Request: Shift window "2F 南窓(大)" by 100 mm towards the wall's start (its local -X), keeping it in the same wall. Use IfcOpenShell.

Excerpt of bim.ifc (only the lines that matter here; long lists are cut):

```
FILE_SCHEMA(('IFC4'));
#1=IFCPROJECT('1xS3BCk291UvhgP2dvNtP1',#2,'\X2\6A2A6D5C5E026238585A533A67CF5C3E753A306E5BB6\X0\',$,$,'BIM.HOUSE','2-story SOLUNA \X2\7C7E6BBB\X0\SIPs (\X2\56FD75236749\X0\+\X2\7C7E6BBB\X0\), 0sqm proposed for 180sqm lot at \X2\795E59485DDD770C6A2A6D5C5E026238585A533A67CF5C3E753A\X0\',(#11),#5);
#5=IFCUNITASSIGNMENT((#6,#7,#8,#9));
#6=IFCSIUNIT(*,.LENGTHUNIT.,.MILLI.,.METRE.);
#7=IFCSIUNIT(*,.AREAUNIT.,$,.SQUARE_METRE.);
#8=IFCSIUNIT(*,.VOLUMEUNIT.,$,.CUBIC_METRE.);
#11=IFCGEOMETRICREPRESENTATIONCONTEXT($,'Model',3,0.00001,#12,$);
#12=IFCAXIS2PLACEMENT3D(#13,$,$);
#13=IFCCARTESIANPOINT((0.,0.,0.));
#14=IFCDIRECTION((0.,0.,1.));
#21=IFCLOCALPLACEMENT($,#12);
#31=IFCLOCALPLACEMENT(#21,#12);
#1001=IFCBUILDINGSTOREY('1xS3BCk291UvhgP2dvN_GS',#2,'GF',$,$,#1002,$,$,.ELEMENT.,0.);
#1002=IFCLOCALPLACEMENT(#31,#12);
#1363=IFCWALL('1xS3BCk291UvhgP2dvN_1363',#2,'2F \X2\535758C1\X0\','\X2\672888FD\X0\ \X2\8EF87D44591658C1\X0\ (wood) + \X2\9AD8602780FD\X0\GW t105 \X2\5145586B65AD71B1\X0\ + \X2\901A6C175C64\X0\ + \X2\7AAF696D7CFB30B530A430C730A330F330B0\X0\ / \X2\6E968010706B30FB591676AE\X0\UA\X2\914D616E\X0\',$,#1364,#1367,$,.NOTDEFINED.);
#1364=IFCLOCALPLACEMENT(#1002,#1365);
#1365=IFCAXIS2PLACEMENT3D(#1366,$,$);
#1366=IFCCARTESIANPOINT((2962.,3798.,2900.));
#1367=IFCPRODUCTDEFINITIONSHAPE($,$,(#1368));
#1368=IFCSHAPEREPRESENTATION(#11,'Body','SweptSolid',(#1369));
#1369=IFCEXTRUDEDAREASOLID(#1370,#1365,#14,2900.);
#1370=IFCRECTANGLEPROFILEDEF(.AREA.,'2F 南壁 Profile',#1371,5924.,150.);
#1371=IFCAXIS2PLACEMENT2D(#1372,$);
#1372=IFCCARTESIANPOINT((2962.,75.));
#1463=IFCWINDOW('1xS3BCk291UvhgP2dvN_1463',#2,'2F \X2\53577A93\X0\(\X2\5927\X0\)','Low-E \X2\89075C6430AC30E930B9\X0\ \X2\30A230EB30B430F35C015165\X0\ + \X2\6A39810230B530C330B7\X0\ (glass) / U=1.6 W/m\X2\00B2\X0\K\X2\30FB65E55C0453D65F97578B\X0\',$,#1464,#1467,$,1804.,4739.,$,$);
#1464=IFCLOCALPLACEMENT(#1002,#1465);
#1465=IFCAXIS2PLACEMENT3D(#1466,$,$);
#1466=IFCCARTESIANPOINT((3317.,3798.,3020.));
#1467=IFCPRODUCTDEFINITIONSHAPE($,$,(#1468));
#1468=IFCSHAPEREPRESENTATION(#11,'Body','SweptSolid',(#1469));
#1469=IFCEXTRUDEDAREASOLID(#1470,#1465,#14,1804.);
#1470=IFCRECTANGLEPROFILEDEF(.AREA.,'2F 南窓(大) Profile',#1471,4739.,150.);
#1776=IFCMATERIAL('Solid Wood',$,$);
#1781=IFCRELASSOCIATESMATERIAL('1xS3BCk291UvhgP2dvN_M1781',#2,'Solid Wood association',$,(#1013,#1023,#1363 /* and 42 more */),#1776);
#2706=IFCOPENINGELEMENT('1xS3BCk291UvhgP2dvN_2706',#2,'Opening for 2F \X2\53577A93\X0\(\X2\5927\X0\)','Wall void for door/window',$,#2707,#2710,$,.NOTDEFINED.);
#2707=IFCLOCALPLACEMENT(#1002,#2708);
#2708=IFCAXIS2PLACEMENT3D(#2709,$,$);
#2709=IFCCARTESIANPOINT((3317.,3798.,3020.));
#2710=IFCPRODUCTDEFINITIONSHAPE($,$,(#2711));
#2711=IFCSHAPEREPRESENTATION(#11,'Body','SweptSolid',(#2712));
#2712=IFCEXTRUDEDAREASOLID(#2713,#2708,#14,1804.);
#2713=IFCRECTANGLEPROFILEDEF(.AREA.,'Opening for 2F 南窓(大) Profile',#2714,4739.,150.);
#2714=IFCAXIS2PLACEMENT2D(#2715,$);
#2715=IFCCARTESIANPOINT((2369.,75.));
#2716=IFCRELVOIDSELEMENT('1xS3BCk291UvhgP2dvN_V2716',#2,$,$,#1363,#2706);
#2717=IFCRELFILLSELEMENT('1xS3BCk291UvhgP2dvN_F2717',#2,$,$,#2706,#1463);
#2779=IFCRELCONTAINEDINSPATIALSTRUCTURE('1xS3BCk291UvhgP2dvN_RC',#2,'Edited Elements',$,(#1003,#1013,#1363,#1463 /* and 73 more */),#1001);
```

```python
import ifcopenshell
import ifcopenshell.api.geometry
import ifcopenshell.util.placement
import ifcopenshell.util.unit

model = ifcopenshell.open("bim.ifc")
unit_scale = ifcopenshell.util.unit.calculate_unit_scale(model)

window = model.by_id(1463)
opening = window.FillsVoids[0].RelatingOpeningElement
wall = opening.VoidsElements[0].RelatingBuildingElement

wall_matrix = ifcopenshell.util.placement.get_local_placement(wall.ObjectPlacement)
shift = wall_matrix[:3, 0] * -0.1 / unit_scale
before = ifcopenshell.util.placement.get_local_placement(window.ObjectPlacement)[:3, 3].copy()

# The window is not placed relative to its opening, so move both.
for product in (opening, window):
    matrix = ifcopenshell.util.placement.get_local_placement(product.ObjectPlacement)
    matrix[:3, 3] += shift
    ifcopenshell.api.geometry.edit_object_placement(model, product=product, matrix=matrix, is_si=False)

after = ifcopenshell.util.placement.get_local_placement(window.ObjectPlacement)[:3, 3]
print("window moved by", (after - before).round(3) + 0.0)

model.write("bim_rev.ifc")
```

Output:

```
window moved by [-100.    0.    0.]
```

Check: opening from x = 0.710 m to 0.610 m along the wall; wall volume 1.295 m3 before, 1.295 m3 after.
